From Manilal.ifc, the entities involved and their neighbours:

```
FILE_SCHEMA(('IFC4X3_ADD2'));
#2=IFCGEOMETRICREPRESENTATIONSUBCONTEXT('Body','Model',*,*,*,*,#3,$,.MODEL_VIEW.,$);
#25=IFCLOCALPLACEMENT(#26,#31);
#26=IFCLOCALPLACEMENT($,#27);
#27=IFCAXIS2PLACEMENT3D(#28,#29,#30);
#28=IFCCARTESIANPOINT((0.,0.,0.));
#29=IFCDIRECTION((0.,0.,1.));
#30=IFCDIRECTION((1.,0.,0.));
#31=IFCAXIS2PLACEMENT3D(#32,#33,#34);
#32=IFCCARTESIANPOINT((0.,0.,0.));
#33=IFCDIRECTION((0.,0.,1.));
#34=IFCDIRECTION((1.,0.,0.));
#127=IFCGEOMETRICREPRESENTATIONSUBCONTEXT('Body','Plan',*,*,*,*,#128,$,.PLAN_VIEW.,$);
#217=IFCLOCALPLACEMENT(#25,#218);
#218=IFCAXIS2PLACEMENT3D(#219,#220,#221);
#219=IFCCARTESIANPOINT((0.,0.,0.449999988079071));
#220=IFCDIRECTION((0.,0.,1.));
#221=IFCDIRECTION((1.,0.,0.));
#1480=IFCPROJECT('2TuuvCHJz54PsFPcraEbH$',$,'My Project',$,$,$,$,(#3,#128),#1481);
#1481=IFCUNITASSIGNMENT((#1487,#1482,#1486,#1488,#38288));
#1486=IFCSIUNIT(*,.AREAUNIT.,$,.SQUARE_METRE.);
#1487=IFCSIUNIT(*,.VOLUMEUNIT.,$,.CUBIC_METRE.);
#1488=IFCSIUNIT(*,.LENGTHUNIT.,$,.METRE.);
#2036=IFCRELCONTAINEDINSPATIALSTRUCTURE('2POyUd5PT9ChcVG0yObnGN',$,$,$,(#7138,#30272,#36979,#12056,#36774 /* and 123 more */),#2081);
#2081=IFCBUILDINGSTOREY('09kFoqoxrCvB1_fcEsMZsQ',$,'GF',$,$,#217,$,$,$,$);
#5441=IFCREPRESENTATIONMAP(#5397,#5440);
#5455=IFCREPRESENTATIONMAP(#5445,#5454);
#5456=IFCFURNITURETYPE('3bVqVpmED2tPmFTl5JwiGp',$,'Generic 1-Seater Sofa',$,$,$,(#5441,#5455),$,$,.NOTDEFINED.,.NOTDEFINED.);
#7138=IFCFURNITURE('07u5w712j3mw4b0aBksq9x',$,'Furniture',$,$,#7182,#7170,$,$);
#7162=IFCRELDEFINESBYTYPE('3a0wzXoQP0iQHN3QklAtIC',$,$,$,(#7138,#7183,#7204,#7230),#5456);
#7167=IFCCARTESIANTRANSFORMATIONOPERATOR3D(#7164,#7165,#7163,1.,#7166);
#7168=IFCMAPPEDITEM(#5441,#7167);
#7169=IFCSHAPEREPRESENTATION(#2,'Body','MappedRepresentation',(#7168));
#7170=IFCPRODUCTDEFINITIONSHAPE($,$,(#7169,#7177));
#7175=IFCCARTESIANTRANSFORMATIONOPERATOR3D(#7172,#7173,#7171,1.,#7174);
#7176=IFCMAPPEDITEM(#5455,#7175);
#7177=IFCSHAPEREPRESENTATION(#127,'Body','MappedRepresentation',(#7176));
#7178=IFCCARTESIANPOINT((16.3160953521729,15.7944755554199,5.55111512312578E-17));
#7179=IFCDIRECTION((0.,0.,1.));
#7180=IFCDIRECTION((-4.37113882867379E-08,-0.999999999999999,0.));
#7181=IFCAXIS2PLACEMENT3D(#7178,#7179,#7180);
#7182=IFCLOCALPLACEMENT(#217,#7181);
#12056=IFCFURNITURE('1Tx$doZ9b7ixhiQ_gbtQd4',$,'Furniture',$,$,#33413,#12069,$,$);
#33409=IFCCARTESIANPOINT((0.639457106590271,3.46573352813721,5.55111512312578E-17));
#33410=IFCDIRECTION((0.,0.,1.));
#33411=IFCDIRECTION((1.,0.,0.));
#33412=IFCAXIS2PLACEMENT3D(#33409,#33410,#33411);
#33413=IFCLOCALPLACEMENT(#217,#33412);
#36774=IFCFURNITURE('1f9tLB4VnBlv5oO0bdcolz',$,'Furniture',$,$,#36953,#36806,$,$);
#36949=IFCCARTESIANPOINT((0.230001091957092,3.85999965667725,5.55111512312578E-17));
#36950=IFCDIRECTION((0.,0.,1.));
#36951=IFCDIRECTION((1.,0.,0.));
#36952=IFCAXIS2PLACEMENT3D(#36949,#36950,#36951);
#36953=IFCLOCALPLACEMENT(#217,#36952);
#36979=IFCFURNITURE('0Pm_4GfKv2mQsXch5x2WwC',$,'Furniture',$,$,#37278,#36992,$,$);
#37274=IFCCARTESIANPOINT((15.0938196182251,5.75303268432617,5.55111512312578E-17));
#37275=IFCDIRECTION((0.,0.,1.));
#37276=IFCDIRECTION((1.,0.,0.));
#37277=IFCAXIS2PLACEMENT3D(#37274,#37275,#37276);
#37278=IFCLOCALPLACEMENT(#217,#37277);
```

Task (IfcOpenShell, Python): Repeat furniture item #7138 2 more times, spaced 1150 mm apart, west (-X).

```python
import numpy as np
import ifcopenshell
import ifcopenshell.api.geometry
import ifcopenshell.api.root
import ifcopenshell.util.element
import ifcopenshell.util.placement

model = ifcopenshell.open("Manilal.ifc")

source = model.by_guid("07u5w712j3mw4b0aBksq9x")
base = ifcopenshell.util.placement.get_local_placement(source.ObjectPlacement)
step = np.array([-1.0, 0.0, 0.0]) * 1.15

for i in range(1, 3):
    copy = ifcopenshell.api.root.copy_class(model, product=source)
    copy.Representation = ifcopenshell.util.element.copy_deep(
        model, source.Representation, exclude=["IfcGeometricRepresentationContext", "IfcRepresentationMap"]
    )
    matrix = base.copy()
    matrix[:3, 3] += i * step
    print("added at", matrix[:3, 3].round(3) + 0.0)
    ifcopenshell.api.geometry.edit_object_placement(model, product=copy, matrix=matrix, is_si=False)

model.write("Manilal_v2.ifc")
```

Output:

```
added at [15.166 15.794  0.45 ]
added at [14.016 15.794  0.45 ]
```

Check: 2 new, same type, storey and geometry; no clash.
